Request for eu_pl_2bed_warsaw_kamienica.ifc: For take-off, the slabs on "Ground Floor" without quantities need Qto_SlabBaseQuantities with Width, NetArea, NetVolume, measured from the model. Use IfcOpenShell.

First a look at what the model holds.

```python
import ifcopenshell
import ifcopenshell.util.element
import ifcopenshell.util.unit

model = ifcopenshell.open("eu_pl_2bed_warsaw_kamienica.ifc")
print(model.schema)
for unit_type in ("LENGTHUNIT", "AREAUNIT", "VOLUMEUNIT"):
    print(unit_type, ifcopenshell.util.unit.calculate_unit_scale(model, unit_type))
storey = next(s for s in model.by_type("IfcBuildingStorey") if s.Name == "Ground Floor")
slabs = [e for e in ifcopenshell.util.element.get_decomposition(storey) if e.is_a("IfcSlab")]
for e in sorted(slabs, key=lambda e: e.id()):
    print(e.id(), e.is_a(), e.Name, list(ifcopenshell.util.element.get_psets(e, qtos_only=True)), sep=" | ")
```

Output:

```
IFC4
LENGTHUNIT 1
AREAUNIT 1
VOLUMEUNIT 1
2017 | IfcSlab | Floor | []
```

```python
import ifcopenshell
import ifcopenshell.api.pset
import ifcopenshell.geom
import ifcopenshell.util.element
import ifcopenshell.util.shape
import ifcopenshell.util.unit

model = ifcopenshell.open("eu_pl_2bed_warsaw_kamienica.ifc")
unit_scale = ifcopenshell.util.unit.calculate_unit_scale(model)
area_scale = ifcopenshell.util.unit.calculate_unit_scale(model, "AREAUNIT")
volume_scale = ifcopenshell.util.unit.calculate_unit_scale(model, "VOLUMEUNIT")
settings = ifcopenshell.geom.settings()

storey = next(s for s in model.by_type("IfcBuildingStorey") if s.Name == "Ground Floor")
slabs = [e for e in ifcopenshell.util.element.get_decomposition(storey) if e.is_a("IfcSlab")]

for e in sorted(slabs, key=lambda e: e.id()):
    if ifcopenshell.util.element.get_psets(e, qtos_only=True, should_inherit=False):
        continue
    # Geometry comes back in metres, in the element's own axes.
    shape = ifcopenshell.geom.create_shape(settings, e)
    values = {
        "Width": ifcopenshell.util.shape.get_z(shape.geometry) / unit_scale,
        "NetArea": ifcopenshell.util.shape.get_footprint_area(shape.geometry) / area_scale,
        "NetVolume": ifcopenshell.util.shape.get_volume(shape.geometry) / volume_scale,
    }
    qto = ifcopenshell.api.pset.add_qto(model, product=e, name="Qto_SlabBaseQuantities")
    ifcopenshell.api.pset.edit_qto(model, qto=qto, properties=values)
    print(e.id(), {k: round(v, 3) for k, v in values.items()})

model.write("eu_pl_2bed_warsaw_kamienica-out.ifc")
```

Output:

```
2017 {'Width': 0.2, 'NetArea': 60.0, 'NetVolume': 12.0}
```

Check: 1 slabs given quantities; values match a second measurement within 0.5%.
